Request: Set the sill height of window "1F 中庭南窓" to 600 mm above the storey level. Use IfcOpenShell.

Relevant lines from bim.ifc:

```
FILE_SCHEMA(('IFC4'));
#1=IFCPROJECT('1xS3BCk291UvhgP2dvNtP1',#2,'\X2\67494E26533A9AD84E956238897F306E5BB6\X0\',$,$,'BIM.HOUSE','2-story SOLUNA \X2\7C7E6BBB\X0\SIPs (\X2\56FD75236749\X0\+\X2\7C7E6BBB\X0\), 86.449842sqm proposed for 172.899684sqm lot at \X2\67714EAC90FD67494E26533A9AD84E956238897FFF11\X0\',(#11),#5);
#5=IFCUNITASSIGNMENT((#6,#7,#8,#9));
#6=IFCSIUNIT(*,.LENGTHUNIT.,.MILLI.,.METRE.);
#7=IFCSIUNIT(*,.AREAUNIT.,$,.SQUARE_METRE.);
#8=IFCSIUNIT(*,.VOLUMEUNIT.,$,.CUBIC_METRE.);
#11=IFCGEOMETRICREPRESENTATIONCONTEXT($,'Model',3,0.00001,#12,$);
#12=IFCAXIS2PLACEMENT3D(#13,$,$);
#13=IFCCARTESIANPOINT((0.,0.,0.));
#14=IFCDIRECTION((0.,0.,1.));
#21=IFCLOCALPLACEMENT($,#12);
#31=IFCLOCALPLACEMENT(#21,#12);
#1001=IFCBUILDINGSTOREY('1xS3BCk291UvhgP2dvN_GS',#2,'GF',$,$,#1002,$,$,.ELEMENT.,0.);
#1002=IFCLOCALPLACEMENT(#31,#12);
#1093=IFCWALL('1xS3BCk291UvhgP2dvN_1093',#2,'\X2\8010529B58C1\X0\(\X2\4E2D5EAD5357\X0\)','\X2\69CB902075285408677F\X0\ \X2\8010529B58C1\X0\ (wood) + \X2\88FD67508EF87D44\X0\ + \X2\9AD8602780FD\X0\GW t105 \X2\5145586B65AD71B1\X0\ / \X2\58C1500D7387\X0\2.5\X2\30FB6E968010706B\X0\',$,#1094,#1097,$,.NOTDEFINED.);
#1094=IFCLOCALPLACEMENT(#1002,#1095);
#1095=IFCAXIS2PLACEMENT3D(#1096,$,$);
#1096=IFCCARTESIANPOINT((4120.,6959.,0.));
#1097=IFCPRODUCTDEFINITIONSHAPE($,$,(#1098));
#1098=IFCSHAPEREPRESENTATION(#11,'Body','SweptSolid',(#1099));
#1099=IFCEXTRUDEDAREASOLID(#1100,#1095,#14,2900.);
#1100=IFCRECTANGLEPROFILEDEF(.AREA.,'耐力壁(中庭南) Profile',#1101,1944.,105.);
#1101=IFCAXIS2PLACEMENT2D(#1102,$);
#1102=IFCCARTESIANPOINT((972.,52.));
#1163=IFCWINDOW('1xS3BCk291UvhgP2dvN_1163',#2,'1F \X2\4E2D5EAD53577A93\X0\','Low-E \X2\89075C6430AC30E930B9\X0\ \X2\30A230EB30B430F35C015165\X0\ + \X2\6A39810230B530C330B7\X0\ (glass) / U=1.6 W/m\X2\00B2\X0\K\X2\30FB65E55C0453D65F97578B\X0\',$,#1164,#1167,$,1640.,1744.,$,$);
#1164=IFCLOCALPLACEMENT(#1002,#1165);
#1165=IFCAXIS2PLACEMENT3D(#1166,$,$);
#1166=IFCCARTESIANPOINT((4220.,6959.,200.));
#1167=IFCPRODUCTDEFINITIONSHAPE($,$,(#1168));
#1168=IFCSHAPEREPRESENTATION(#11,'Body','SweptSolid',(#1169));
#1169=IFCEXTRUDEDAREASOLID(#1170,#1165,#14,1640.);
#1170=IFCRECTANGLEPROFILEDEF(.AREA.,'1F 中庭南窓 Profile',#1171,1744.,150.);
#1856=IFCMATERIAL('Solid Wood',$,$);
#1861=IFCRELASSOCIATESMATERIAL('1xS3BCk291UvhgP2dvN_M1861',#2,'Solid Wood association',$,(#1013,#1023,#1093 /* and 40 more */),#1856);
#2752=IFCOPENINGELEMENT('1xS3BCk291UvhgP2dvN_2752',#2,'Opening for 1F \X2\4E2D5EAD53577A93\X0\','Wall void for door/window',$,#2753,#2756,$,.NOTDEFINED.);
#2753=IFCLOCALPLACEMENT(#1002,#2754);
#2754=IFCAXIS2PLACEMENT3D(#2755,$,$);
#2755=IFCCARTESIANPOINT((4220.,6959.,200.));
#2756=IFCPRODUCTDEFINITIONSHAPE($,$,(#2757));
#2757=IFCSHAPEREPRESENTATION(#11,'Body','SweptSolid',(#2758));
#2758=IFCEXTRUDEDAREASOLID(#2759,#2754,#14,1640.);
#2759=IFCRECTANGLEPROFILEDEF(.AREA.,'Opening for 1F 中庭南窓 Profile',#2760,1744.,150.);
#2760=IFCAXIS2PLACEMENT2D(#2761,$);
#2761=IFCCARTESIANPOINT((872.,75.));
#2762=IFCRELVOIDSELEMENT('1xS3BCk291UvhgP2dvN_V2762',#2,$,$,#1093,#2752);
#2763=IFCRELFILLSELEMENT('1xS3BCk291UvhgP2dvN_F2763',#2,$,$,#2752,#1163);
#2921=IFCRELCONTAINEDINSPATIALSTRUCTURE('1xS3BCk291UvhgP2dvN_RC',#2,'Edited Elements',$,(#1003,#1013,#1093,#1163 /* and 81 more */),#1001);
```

```python
import numpy as np
import ifcopenshell
import ifcopenshell.api.geometry
import ifcopenshell.geom
import ifcopenshell.util.element
import ifcopenshell.util.placement
import ifcopenshell.util.shape
import ifcopenshell.util.unit

model = ifcopenshell.open("bim.ifc")
unit_scale = ifcopenshell.util.unit.calculate_unit_scale(model)

window = model.by_guid("1xS3BCk291UvhgP2dvN_1163")
opening = window.FillsVoids[0].RelatingOpeningElement
storey = ifcopenshell.util.element.get_container(window, ifc_class="IfcBuildingStorey")
level = ifcopenshell.util.placement.get_local_placement(storey.ObjectPlacement)[2, 3]

# The opening's origin need not be at the sill, so measure its lowest point.
shape = ifcopenshell.geom.create_shape(ifcopenshell.geom.settings(), opening)
bottom = ifcopenshell.util.shape.get_shape_bottom_elevation(shape, shape.geometry) / unit_scale
dz = level + 600.0 - bottom

shift = np.array([0.0, 0.0, dz])
# The window is not placed relative to its opening, so move both.
for product in (opening, window):
    matrix = ifcopenshell.util.placement.get_local_placement(product.ObjectPlacement)
    matrix[:3, 3] += shift
    ifcopenshell.api.geometry.edit_object_placement(model, product=product, matrix=matrix, is_si=False)

print(f"moved by {dz * unit_scale:+.3f} m")

model.write("bim_edited.ifc")
```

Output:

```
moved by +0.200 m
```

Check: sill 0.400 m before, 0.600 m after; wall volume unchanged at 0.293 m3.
